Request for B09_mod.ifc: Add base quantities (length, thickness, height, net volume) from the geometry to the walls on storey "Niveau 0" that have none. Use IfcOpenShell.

First a look at what the model holds.

```python
import ifcopenshell
import ifcopenshell.util.element
import ifcopenshell.util.unit

model = ifcopenshell.open("B09_mod.ifc")
print(model.schema)
for unit_type in ("LENGTHUNIT", "AREAUNIT", "VOLUMEUNIT"):
    print(unit_type, ifcopenshell.util.unit.calculate_unit_scale(model, unit_type))
storey = next(s for s in model.by_type("IfcBuildingStorey") if s.Name == "Niveau 0")
walls = [e for e in ifcopenshell.util.element.get_decomposition(storey) if e.is_a("IfcWall")]
for e in sorted(walls, key=lambda e: e.id()):
    print(e.id(), e.is_a(), e.Name, list(ifcopenshell.util.element.get_psets(e, qtos_only=True)), sep=" | ")
```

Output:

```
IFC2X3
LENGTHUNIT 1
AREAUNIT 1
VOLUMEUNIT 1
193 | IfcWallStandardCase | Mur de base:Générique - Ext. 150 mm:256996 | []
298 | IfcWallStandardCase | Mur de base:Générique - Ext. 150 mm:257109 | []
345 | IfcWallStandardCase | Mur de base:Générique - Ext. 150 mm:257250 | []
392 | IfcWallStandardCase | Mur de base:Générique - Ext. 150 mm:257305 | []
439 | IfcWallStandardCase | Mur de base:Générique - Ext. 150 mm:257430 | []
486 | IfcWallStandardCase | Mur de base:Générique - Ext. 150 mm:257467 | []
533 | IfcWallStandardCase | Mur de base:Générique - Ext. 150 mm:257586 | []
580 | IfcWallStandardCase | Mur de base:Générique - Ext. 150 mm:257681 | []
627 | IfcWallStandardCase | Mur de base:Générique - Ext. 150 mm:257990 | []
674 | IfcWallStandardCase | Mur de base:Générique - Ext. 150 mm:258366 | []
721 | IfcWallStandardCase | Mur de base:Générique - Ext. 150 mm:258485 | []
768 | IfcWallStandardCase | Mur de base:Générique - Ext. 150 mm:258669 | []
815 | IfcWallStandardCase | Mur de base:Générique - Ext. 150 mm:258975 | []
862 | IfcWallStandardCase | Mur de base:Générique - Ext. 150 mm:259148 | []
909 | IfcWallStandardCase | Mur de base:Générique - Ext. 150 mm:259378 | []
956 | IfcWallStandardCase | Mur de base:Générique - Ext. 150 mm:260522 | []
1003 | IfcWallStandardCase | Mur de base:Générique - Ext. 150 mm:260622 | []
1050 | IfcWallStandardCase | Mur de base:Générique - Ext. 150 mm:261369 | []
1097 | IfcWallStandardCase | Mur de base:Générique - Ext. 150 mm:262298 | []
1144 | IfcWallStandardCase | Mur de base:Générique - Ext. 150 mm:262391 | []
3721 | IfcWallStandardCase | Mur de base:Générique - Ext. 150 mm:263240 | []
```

```python
import ifcopenshell
import ifcopenshell.api.pset
import ifcopenshell.geom
import ifcopenshell.util.element
import ifcopenshell.util.shape
import ifcopenshell.util.unit

model = ifcopenshell.open("B09_mod.ifc")
unit_scale = ifcopenshell.util.unit.calculate_unit_scale(model)
volume_scale = ifcopenshell.util.unit.calculate_unit_scale(model, "VOLUMEUNIT")
settings = ifcopenshell.geom.settings()

storey = next(s for s in model.by_type("IfcBuildingStorey") if s.Name == "Niveau 0")
walls = [e for e in ifcopenshell.util.element.get_decomposition(storey) if e.is_a("IfcWall")]

for e in sorted(walls, key=lambda e: e.id()):
    if ifcopenshell.util.element.get_psets(e, qtos_only=True, should_inherit=False):
        continue
    # Geometry comes back in metres, in the element's own axes.
    shape = ifcopenshell.geom.create_shape(settings, e)
    values = {
        "Length": ifcopenshell.util.shape.get_x(shape.geometry) / unit_scale,
        "Width": ifcopenshell.util.shape.get_y(shape.geometry) / unit_scale,
        "Height": ifcopenshell.util.shape.get_z(shape.geometry) / unit_scale,
        "NetVolume": ifcopenshell.util.shape.get_volume(shape.geometry) / volume_scale,
    }
    qto = ifcopenshell.api.pset.add_qto(model, product=e, name="BaseQuantities")
    ifcopenshell.api.pset.edit_qto(model, qto=qto, properties=values)
    print(e.id(), {k: round(v, 3) for k, v in values.items()})

model.write("B09_mod_updated.ifc")
```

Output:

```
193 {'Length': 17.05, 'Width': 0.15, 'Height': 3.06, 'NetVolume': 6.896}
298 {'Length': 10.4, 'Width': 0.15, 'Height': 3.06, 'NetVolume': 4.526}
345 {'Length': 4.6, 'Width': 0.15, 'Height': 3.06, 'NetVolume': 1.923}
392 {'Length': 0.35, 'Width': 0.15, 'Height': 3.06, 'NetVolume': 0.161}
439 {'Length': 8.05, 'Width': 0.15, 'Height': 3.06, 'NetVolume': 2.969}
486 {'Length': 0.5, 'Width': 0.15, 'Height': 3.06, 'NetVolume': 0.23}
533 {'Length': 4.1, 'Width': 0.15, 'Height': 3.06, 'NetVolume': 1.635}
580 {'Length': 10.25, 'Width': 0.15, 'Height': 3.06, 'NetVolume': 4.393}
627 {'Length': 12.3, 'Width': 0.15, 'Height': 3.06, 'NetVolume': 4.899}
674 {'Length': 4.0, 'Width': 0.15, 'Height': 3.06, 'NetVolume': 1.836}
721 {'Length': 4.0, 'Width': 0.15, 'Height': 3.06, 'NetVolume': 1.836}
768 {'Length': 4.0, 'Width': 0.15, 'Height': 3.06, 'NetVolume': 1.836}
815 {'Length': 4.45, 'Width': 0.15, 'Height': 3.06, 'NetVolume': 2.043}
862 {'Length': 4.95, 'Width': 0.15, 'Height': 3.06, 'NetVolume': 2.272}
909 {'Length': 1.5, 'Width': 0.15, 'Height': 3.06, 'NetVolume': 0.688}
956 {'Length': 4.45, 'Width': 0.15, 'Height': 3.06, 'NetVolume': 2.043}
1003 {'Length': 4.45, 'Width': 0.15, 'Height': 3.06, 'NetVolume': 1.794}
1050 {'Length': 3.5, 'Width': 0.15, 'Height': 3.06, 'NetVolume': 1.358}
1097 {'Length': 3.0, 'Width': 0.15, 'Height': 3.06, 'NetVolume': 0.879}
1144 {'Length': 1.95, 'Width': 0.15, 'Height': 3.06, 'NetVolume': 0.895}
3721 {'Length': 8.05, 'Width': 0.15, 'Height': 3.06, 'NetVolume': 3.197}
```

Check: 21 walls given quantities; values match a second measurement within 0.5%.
